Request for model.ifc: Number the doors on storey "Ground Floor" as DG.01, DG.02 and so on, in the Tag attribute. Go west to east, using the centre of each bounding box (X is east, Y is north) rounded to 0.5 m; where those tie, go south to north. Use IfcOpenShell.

First a look at what the model holds.

```python
import ifcopenshell
import ifcopenshell.util.element
import ifcopenshell.util.placement

model = ifcopenshell.open("model.ifc")
print(model.schema)
storey = next(s for s in model.by_type("IfcBuildingStorey") if s.Name == "Ground Floor")
doors = [e for e in ifcopenshell.util.element.get_decomposition(storey) if e.is_a("IfcDoor")]
for e in sorted(doors, key=lambda e: e.id()):
    origin = ifcopenshell.util.placement.get_local_placement(e.ObjectPlacement)[:3, 3]
    print(e.id(), e.Tag, e.Name, origin.round(2) + 0.0, sep=" | ")
```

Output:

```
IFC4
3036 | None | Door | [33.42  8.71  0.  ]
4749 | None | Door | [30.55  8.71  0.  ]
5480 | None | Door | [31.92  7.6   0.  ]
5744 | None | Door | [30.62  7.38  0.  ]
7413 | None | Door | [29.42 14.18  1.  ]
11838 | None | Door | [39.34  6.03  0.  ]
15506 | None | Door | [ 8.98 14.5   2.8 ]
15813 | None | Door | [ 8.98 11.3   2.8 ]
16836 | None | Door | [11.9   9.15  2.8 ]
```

```python
import ifcopenshell
import ifcopenshell.geom
import ifcopenshell.util.element
import ifcopenshell.util.shape

model = ifcopenshell.open("model.ifc")
settings = ifcopenshell.geom.settings()
settings.set("use-world-coords", True)


def centre(element):
    shape = ifcopenshell.geom.create_shape(settings, element)
    return ifcopenshell.util.shape.get_bbox_centroid(shape.geometry)


storey = next(s for s in model.by_type("IfcBuildingStorey") if s.Name == "Ground Floor")
doors = [e for e in ifcopenshell.util.element.get_decomposition(storey) if e.is_a("IfcDoor")]

# Insertion points can sit at a corner or the storey origin, so sort by the geometry (in metres).
centres = {e: centre(e) for e in doors}
doors.sort(key=lambda e: (round(centres[e][0] / 0.5), centres[e][1]))

for i, e in enumerate(doors, start=1):
    number = f"DG.{i:02d}"
    e.Tag = number
    print(e.id(), number)

model.write("model_v2.ifc")
```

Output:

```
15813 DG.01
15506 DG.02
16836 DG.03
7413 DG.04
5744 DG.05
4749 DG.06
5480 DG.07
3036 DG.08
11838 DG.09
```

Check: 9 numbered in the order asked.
